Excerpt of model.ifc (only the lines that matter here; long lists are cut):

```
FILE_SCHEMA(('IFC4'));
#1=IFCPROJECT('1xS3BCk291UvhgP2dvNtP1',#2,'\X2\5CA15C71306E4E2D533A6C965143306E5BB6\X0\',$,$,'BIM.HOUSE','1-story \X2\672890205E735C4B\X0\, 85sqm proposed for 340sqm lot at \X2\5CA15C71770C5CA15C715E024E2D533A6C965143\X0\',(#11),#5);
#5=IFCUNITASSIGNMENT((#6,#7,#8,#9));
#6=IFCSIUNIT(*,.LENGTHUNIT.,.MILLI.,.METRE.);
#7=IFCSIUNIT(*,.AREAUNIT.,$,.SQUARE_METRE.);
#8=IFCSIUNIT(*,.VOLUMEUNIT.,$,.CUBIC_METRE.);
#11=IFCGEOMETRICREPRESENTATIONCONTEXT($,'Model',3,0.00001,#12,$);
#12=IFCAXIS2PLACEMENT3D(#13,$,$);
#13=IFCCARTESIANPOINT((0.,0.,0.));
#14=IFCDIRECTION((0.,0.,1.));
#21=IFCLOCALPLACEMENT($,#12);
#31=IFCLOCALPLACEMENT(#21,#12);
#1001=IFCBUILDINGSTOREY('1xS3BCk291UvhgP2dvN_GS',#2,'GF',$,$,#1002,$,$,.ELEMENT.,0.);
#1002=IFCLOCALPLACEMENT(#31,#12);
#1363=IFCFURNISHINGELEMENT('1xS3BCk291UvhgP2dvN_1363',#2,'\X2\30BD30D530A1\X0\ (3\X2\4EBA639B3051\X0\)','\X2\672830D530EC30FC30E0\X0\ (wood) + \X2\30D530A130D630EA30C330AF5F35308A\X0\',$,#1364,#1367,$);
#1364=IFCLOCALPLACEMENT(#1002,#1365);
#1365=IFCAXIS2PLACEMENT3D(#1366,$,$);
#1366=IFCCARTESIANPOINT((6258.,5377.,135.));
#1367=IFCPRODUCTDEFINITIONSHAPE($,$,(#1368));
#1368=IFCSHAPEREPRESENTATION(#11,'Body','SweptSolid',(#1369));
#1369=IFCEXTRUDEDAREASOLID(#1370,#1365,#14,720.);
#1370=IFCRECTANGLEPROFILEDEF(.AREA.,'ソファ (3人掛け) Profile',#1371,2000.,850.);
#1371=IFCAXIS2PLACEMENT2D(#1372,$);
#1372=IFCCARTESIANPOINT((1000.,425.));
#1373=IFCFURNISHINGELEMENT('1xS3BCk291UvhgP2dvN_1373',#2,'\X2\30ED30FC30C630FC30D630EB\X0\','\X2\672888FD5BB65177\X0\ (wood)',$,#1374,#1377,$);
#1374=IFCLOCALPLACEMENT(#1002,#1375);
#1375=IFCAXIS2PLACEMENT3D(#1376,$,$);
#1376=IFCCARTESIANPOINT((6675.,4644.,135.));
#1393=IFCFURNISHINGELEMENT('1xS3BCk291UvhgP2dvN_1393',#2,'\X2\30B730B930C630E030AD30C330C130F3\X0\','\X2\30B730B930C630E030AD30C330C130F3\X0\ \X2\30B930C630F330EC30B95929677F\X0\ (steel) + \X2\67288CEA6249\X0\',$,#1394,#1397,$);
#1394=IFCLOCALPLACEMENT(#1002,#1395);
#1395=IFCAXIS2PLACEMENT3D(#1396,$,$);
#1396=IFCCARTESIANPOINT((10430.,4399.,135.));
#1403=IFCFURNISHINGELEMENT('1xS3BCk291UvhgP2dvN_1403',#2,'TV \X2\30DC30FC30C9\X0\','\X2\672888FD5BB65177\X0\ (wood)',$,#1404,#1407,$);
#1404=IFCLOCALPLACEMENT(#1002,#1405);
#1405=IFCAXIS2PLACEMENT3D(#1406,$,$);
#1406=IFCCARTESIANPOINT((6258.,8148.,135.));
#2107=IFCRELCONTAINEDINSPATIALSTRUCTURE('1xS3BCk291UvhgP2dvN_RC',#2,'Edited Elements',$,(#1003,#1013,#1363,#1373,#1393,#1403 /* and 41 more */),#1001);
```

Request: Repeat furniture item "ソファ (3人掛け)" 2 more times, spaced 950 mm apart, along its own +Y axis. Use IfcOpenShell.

```python
import ifcopenshell
import ifcopenshell.api.geometry
import ifcopenshell.api.root
import ifcopenshell.util.element
import ifcopenshell.util.placement
import ifcopenshell.util.unit

model = ifcopenshell.open("model.ifc")
unit_scale = ifcopenshell.util.unit.calculate_unit_scale(model)


def reuse_history(source, copy):
    """copy_class also copies each property set's owner history, people and application; keep the originals."""
    for rel in copy.IsDefinedBy:
        if rel.is_a("IfcRelDefinesByProperties") and (history := rel.RelatingPropertyDefinition.OwnerHistory):
            rel.RelatingPropertyDefinition.OwnerHistory = source.OwnerHistory
            ifcopenshell.util.element.remove_deep2(model, history)


source = model.by_guid("1xS3BCk291UvhgP2dvN_1363")
base = ifcopenshell.util.placement.get_local_placement(source.ObjectPlacement)
step = base[:3, 1] * 0.95 / unit_scale

for i in range(1, 3):
    copy = ifcopenshell.api.root.copy_class(model, product=source)
    copy.Representation = ifcopenshell.util.element.copy_deep(
        model, source.Representation, exclude=["IfcGeometricRepresentationContext", "IfcRepresentationMap"]
    )
    reuse_history(source, copy)
    matrix = base.copy()
    matrix[:3, 3] += i * step
    print("added at", matrix[:3, 3].round(3) + 0.0)
    ifcopenshell.api.geometry.edit_object_placement(model, product=copy, matrix=matrix, is_si=False)

model.write("model_v2.ifc")
```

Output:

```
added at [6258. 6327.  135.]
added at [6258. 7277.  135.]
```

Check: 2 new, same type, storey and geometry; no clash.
